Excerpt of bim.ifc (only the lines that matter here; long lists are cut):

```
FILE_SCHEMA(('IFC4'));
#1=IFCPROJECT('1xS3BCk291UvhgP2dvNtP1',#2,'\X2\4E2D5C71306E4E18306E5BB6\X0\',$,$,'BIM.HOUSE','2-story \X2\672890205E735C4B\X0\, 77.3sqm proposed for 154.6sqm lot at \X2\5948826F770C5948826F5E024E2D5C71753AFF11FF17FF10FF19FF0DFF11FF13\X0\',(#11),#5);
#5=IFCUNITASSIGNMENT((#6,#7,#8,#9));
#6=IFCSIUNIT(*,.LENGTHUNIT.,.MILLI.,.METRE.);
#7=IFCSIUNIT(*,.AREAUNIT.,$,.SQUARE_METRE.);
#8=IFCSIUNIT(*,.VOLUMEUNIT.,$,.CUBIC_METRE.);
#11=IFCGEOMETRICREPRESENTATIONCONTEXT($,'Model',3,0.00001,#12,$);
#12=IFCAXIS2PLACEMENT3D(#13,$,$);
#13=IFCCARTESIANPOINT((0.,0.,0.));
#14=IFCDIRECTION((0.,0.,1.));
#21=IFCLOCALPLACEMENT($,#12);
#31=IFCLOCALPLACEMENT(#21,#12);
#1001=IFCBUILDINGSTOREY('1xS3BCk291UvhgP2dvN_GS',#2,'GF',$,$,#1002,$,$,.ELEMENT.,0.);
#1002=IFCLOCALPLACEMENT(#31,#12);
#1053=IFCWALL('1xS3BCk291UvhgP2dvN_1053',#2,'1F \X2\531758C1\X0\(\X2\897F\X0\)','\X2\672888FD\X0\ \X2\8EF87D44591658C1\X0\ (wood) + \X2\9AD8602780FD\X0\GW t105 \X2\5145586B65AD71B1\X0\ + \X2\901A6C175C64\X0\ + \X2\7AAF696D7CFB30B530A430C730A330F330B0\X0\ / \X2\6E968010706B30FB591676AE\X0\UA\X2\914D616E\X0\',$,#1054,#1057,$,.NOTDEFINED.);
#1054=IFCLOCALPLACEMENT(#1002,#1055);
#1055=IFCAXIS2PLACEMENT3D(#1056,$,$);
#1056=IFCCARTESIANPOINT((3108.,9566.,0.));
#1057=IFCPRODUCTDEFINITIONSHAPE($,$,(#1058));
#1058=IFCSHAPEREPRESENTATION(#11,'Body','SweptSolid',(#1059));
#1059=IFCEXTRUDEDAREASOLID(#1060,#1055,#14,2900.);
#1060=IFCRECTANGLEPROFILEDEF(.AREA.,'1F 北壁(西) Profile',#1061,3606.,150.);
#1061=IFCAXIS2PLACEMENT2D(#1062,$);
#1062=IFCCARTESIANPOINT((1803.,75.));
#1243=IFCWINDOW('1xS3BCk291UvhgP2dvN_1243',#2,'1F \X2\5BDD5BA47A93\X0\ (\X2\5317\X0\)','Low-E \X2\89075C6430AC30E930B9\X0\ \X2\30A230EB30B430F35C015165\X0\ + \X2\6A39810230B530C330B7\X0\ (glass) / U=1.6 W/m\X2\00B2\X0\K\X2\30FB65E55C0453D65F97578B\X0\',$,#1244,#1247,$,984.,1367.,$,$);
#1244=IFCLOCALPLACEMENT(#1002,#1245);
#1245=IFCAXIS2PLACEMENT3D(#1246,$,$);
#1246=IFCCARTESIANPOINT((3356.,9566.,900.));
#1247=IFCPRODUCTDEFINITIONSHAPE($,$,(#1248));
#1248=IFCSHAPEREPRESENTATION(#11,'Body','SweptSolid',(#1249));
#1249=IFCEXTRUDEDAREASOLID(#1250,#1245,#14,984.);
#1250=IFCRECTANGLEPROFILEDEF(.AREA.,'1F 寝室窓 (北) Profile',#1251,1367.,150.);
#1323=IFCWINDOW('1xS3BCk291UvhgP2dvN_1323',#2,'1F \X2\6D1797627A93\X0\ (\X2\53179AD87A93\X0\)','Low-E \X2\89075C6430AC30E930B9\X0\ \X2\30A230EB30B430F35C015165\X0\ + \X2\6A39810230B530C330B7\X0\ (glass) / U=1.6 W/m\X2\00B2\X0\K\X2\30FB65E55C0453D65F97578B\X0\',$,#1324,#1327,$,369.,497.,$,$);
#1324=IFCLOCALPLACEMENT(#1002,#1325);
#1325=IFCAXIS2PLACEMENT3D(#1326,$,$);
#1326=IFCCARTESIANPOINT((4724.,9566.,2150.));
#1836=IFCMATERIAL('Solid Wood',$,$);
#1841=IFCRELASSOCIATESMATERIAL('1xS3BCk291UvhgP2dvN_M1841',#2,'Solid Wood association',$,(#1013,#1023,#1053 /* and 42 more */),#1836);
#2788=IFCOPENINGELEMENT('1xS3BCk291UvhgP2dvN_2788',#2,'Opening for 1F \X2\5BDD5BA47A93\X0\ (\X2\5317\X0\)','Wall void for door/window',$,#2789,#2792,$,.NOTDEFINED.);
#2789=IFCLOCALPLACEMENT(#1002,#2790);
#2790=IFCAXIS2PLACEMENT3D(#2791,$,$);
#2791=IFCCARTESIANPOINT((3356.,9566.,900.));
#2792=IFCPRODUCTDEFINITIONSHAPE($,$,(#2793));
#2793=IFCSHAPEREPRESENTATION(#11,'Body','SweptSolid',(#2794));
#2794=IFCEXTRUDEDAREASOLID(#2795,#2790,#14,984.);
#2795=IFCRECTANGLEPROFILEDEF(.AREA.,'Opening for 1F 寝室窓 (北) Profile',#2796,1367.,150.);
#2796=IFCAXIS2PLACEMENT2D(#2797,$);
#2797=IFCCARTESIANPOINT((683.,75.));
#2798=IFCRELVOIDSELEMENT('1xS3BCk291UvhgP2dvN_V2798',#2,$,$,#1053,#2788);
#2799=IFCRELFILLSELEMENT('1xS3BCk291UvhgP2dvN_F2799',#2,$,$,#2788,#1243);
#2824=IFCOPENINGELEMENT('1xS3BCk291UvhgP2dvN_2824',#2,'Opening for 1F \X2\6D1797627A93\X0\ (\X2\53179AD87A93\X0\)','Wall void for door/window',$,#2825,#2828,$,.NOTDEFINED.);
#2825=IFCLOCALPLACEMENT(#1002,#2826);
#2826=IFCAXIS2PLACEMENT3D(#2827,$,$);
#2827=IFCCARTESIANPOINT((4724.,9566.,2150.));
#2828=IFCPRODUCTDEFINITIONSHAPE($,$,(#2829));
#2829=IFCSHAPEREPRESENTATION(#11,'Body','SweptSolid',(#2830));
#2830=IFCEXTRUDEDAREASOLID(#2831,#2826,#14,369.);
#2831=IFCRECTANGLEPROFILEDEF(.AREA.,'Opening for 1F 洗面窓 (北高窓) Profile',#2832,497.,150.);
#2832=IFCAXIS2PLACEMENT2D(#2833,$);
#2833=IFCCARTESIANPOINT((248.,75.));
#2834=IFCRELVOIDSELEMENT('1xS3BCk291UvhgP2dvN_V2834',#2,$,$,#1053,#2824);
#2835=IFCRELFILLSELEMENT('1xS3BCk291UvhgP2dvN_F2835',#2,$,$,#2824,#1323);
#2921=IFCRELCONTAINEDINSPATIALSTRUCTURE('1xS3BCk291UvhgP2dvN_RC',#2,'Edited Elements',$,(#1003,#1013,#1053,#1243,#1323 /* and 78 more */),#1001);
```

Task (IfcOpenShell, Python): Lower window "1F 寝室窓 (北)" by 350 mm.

```python
import numpy as np
import ifcopenshell
import ifcopenshell.api.geometry
import ifcopenshell.util.placement
import ifcopenshell.util.unit

model = ifcopenshell.open("bim.ifc")
unit_scale = ifcopenshell.util.unit.calculate_unit_scale(model)

window = model.by_id(1243)
opening = window.FillsVoids[0].RelatingOpeningElement
dz = -0.35 / unit_scale

shift = np.array([0.0, 0.0, dz])
# The window is not placed relative to its opening, so move both.
for product in (opening, window):
    matrix = ifcopenshell.util.placement.get_local_placement(product.ObjectPlacement)
    matrix[:3, 3] += shift
    ifcopenshell.api.geometry.edit_object_placement(model, product=product, matrix=matrix, is_si=False)

print(f"moved by {dz * unit_scale:+.3f} m")

model.write("bim_edited.ifc")
```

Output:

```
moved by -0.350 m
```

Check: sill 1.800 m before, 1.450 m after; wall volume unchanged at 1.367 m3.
